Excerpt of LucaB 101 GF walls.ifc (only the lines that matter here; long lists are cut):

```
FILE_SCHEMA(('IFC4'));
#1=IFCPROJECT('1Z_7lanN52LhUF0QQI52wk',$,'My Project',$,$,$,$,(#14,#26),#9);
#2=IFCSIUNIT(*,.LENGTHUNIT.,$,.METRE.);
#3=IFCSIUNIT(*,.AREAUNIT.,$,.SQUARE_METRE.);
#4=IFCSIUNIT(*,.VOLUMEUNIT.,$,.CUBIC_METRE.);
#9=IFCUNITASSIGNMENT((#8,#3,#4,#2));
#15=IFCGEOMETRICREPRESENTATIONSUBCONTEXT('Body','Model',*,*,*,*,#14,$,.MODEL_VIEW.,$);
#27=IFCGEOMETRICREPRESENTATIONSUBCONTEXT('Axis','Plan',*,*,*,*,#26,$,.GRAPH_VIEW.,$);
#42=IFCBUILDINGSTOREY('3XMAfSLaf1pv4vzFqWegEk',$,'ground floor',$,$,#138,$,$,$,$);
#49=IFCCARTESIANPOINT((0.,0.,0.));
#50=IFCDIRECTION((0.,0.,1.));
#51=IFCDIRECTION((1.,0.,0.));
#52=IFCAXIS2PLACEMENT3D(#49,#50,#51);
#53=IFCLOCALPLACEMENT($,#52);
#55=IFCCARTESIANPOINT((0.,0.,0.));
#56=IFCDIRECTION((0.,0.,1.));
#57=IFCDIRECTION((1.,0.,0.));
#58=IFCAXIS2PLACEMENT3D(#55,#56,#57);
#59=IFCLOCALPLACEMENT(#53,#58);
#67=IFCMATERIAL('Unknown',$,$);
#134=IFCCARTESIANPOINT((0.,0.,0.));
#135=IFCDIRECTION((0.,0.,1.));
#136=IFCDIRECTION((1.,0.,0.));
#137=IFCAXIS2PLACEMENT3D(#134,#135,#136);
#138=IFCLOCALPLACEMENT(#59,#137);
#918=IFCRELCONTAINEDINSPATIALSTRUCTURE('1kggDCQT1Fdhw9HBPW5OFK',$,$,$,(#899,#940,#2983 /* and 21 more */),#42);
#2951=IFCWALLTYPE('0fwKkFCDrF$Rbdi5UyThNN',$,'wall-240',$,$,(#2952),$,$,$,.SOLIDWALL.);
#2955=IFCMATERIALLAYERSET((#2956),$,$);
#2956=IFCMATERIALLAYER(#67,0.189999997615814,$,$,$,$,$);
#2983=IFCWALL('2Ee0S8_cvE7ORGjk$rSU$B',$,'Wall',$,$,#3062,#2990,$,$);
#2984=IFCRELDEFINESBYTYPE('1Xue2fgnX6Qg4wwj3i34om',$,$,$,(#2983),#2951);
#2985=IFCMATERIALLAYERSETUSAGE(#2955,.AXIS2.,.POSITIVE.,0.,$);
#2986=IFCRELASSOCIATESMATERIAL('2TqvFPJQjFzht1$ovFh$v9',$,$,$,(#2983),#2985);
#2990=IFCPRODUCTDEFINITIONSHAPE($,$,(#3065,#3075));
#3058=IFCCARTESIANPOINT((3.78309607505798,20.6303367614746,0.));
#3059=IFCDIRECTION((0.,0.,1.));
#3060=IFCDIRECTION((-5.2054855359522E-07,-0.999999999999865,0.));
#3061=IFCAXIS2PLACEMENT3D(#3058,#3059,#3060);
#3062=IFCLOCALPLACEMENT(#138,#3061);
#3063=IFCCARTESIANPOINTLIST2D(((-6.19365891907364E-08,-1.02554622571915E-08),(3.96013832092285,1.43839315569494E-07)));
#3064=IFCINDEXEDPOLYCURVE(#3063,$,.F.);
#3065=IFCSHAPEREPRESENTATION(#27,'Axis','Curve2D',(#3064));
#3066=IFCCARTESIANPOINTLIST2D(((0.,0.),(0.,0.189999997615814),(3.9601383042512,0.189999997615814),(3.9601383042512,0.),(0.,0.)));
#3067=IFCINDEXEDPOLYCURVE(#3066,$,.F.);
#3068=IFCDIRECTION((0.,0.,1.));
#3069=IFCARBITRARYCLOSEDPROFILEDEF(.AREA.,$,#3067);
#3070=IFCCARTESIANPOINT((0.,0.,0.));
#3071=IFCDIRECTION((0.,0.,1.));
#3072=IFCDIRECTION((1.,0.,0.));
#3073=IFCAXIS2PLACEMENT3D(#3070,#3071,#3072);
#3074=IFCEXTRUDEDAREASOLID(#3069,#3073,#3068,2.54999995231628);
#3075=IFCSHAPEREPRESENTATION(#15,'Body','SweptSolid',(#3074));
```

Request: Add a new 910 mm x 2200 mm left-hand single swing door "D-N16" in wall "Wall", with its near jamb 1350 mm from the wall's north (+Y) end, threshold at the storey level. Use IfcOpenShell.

```python
import numpy as np
import ifcopenshell
import ifcopenshell.api.feature
import ifcopenshell.api.geometry
import ifcopenshell.api.root
import ifcopenshell.api.spatial
import ifcopenshell.geom
import ifcopenshell.util.element
import ifcopenshell.util.placement
import ifcopenshell.util.representation
import ifcopenshell.util.shape
import ifcopenshell.util.unit

model = ifcopenshell.open("LucaB 101 GF walls.ifc")
unit_scale = ifcopenshell.util.unit.calculate_unit_scale(model)
settings = ifcopenshell.geom.settings()


def volume(element):
    """Net volume in cubic metres, openings subtracted."""
    shape = ifcopenshell.geom.create_shape(settings, element)
    return ifcopenshell.util.shape.get_volume(shape.geometry)


wall = model.by_id(2983)
storey = ifcopenshell.util.element.get_container(wall, ifc_class="IfcBuildingStorey")
context = ifcopenshell.util.representation.get_context(model, "Model", "Body", "MODEL_VIEW")
before = volume(wall)

width, height, from_end, sill = 0.91, 2.2, 1.35, 0.0  # metres

# The wall runs along its own X axis, and the end named is its -X end.
wall_shape = ifcopenshell.geom.create_shape(settings, wall)
x, y, z = ifcopenshell.util.shape.get_vertices(wall_shape.geometry).T
start = x.min() + from_end
face, thickness = float(y.min()), float(y.max() - y.min())
wall_matrix = ifcopenshell.util.placement.get_local_placement(wall.ObjectPlacement)
level = ifcopenshell.util.placement.get_local_placement(storey.ObjectPlacement)[2, 3]


def in_wall(x, y):
    """Placement at x, y metres in the wall's axes, at sill height."""
    matrix = wall_matrix.copy()
    matrix[:, 3] = wall_matrix @ np.array([x / unit_scale, y / unit_scale, 0.0, 1.0])
    matrix[2, 3] = level + sill / unit_scale
    return matrix


# Opening: a box that overshoots both wall faces by 50 mm.
opening = ifcopenshell.api.root.create_entity(model, ifc_class="IfcOpeningElement", predefined_type="OPENING")
box = ifcopenshell.api.geometry.add_wall_representation(
    model, context=context, length=width, height=height, thickness=thickness + 0.1
)
ifcopenshell.api.geometry.assign_representation(model, product=opening, representation=box)
ifcopenshell.api.geometry.edit_object_placement(model, product=opening, matrix=in_wall(start, face - 0.05), is_si=False)
ifcopenshell.api.feature.add_feature(model, feature=opening, element=wall)

door = ifcopenshell.api.root.create_entity(model, ifc_class="IfcDoor", name="D-N16", predefined_type="DOOR")
door.OverallWidth, door.OverallHeight = width / unit_scale, height / unit_scale
door.OperationType = "SINGLE_SWING_LEFT"
body = ifcopenshell.api.geometry.add_door_representation(
    model,
    context=context,
    overall_width=door.OverallWidth,
    overall_height=door.OverallHeight,
    operation_type="SINGLE_SWING_LEFT",
    lining_properties={"LiningDepth": thickness / unit_scale, "ThresholdDepth": thickness / unit_scale},
)
ifcopenshell.api.geometry.assign_representation(model, product=door, representation=body)
ifcopenshell.api.spatial.assign_container(model, products=[door], relating_structure=storey)
ifcopenshell.api.feature.add_filling(model, opening=opening, element=door)

# The lining spans the wall, so the door starts at the wall face.
ifcopenshell.api.geometry.edit_object_placement(model, product=door, matrix=in_wall(start, face), is_si=False)

after = volume(wall)

print(f"wall volume {before:.3f} -> {after:.3f} m3")

model.write("LucaB 101 GF walls_updated.ifc")
```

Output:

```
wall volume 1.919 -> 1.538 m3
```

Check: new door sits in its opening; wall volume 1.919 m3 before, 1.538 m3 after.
